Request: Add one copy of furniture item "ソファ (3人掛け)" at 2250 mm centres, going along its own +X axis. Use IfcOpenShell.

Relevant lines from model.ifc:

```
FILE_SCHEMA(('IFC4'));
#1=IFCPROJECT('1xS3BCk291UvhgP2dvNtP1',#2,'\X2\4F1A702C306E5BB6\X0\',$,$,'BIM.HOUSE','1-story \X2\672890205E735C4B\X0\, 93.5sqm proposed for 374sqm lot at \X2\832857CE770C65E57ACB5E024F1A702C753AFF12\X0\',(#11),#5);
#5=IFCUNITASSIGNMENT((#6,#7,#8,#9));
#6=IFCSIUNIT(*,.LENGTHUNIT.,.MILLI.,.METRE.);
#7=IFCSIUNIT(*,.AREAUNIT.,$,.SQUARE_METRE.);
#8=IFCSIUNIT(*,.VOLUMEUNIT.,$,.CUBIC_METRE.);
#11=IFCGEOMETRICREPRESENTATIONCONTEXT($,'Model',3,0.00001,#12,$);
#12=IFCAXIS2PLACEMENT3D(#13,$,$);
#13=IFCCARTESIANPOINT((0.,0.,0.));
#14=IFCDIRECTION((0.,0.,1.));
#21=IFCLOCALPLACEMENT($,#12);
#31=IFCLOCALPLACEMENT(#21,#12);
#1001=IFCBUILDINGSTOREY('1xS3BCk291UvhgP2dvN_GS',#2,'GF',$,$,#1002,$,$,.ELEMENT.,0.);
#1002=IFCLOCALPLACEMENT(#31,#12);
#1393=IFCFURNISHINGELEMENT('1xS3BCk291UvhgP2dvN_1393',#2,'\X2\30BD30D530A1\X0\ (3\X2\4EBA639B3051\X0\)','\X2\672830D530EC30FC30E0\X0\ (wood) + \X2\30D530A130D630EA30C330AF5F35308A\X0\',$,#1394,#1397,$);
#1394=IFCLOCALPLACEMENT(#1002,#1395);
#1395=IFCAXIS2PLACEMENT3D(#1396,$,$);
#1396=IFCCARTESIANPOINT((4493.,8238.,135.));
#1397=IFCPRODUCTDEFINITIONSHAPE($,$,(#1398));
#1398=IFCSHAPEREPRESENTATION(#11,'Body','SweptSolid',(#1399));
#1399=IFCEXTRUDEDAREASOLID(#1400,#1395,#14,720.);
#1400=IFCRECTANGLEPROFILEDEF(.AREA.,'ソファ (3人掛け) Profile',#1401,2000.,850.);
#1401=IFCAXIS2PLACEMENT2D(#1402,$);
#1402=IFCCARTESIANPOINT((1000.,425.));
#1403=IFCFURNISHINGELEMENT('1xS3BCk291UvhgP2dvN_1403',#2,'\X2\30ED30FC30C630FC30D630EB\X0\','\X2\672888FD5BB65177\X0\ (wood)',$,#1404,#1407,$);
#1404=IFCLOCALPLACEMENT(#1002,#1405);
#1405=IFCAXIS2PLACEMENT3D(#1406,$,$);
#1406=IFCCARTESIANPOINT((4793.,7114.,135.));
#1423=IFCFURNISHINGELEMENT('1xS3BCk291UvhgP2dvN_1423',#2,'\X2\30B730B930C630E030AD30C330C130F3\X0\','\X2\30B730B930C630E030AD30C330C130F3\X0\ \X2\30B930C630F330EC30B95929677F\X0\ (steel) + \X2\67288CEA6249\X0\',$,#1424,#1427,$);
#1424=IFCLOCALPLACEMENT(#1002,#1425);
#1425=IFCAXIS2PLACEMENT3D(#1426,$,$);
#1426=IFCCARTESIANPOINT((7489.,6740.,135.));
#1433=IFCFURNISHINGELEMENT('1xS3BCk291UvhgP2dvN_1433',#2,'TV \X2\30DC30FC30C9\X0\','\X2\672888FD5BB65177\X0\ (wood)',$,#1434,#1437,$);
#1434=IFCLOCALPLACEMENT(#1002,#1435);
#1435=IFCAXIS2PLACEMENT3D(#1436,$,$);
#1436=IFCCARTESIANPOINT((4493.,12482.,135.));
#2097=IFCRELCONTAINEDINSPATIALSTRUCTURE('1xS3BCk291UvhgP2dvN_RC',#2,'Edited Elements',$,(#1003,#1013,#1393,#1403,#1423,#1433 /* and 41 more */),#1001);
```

```python
import ifcopenshell
import ifcopenshell.api.geometry
import ifcopenshell.api.root
import ifcopenshell.util.element
import ifcopenshell.util.placement

model = ifcopenshell.open("model.ifc")


def reuse_history(source, copy):
    """copy_class also copies each property set's owner history, people and application; keep the originals."""
    for rel in copy.IsDefinedBy:
        if rel.is_a("IfcRelDefinesByProperties") and (history := rel.RelatingPropertyDefinition.OwnerHistory):
            rel.RelatingPropertyDefinition.OwnerHistory = source.OwnerHistory
            ifcopenshell.util.element.remove_deep2(model, history)


source = model.by_guid("1xS3BCk291UvhgP2dvN_1393")
base = ifcopenshell.util.placement.get_local_placement(source.ObjectPlacement)
step = base[:3, 0] * 2250.0

for i in range(1, 2):
    copy = ifcopenshell.api.root.copy_class(model, product=source)
    copy.Representation = ifcopenshell.util.element.copy_deep(
        model, source.Representation, exclude=["IfcGeometricRepresentationContext", "IfcRepresentationMap"]
    )
    reuse_history(source, copy)
    matrix = base.copy()
    matrix[:3, 3] += i * step
    print("added at", matrix[:3, 3].round(3) + 0.0)
    ifcopenshell.api.geometry.edit_object_placement(model, product=copy, matrix=matrix, is_si=False)

model.write("model_edited.ifc")
```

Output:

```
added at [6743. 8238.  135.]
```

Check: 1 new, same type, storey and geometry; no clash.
